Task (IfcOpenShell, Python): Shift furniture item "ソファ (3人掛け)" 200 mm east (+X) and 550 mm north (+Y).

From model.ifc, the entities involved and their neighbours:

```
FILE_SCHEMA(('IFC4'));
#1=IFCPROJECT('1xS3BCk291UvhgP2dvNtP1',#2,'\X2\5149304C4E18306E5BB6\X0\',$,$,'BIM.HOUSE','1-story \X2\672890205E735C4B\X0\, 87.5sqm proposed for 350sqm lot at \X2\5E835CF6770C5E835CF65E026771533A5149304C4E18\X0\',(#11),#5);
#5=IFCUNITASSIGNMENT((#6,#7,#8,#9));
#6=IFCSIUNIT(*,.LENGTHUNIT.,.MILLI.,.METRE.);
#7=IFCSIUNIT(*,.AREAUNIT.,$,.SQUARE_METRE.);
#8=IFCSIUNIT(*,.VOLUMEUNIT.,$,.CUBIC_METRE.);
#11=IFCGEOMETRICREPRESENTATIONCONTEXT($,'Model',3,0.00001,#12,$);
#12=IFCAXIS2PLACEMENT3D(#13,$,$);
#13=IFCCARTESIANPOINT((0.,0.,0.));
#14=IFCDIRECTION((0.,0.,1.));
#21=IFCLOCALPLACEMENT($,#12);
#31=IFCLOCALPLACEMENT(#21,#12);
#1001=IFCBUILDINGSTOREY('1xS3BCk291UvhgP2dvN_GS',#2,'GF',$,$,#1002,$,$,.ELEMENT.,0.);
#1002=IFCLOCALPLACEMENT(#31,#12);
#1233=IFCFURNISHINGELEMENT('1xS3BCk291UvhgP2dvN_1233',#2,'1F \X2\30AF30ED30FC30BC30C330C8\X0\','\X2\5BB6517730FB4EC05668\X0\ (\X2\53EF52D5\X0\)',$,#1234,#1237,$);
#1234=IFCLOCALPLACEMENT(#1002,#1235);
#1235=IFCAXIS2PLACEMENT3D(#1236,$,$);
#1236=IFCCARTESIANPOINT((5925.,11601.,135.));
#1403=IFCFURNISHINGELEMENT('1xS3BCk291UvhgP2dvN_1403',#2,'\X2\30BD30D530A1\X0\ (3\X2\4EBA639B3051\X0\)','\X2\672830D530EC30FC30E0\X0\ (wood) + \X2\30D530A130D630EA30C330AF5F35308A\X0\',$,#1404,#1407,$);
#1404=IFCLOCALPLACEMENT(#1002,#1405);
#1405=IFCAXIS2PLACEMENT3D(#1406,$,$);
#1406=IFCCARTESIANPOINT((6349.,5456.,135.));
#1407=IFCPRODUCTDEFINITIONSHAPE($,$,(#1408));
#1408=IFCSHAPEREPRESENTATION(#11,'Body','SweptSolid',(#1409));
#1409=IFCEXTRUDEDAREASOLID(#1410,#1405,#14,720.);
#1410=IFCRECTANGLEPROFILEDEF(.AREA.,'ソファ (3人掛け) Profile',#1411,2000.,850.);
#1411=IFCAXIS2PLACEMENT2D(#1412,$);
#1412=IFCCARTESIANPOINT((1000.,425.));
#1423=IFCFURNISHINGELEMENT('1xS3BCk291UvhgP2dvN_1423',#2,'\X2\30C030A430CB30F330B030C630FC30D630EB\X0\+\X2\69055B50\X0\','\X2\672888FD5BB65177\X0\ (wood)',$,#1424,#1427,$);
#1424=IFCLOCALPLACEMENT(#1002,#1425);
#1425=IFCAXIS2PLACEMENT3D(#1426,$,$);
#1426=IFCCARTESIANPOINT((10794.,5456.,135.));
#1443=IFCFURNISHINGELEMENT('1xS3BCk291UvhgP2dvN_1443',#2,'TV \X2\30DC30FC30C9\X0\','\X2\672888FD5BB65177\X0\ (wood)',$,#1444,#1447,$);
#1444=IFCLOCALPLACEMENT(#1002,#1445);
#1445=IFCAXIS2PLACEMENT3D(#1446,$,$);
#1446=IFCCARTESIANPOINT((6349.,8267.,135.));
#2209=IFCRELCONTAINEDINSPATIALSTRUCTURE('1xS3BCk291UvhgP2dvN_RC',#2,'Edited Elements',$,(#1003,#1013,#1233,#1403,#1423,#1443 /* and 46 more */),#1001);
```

```python
import ifcopenshell
import ifcopenshell.api.geometry
import ifcopenshell.util.placement

model = ifcopenshell.open("model.ifc")

item = model.by_id(1403)
matrix = ifcopenshell.util.placement.get_local_placement(item.ObjectPlacement)
matrix[0, 3] += 200.0
matrix[1, 3] += 550.0
ifcopenshell.api.geometry.edit_object_placement(model, product=item, matrix=matrix, is_si=False)

print(ifcopenshell.util.placement.get_local_placement(item.ObjectPlacement).round(3) + 0.0)

model.write("model_rev.ifc")
```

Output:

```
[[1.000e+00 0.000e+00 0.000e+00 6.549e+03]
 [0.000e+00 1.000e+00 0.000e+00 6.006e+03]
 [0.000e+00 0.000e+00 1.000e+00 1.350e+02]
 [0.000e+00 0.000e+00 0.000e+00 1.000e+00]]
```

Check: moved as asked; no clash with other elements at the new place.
